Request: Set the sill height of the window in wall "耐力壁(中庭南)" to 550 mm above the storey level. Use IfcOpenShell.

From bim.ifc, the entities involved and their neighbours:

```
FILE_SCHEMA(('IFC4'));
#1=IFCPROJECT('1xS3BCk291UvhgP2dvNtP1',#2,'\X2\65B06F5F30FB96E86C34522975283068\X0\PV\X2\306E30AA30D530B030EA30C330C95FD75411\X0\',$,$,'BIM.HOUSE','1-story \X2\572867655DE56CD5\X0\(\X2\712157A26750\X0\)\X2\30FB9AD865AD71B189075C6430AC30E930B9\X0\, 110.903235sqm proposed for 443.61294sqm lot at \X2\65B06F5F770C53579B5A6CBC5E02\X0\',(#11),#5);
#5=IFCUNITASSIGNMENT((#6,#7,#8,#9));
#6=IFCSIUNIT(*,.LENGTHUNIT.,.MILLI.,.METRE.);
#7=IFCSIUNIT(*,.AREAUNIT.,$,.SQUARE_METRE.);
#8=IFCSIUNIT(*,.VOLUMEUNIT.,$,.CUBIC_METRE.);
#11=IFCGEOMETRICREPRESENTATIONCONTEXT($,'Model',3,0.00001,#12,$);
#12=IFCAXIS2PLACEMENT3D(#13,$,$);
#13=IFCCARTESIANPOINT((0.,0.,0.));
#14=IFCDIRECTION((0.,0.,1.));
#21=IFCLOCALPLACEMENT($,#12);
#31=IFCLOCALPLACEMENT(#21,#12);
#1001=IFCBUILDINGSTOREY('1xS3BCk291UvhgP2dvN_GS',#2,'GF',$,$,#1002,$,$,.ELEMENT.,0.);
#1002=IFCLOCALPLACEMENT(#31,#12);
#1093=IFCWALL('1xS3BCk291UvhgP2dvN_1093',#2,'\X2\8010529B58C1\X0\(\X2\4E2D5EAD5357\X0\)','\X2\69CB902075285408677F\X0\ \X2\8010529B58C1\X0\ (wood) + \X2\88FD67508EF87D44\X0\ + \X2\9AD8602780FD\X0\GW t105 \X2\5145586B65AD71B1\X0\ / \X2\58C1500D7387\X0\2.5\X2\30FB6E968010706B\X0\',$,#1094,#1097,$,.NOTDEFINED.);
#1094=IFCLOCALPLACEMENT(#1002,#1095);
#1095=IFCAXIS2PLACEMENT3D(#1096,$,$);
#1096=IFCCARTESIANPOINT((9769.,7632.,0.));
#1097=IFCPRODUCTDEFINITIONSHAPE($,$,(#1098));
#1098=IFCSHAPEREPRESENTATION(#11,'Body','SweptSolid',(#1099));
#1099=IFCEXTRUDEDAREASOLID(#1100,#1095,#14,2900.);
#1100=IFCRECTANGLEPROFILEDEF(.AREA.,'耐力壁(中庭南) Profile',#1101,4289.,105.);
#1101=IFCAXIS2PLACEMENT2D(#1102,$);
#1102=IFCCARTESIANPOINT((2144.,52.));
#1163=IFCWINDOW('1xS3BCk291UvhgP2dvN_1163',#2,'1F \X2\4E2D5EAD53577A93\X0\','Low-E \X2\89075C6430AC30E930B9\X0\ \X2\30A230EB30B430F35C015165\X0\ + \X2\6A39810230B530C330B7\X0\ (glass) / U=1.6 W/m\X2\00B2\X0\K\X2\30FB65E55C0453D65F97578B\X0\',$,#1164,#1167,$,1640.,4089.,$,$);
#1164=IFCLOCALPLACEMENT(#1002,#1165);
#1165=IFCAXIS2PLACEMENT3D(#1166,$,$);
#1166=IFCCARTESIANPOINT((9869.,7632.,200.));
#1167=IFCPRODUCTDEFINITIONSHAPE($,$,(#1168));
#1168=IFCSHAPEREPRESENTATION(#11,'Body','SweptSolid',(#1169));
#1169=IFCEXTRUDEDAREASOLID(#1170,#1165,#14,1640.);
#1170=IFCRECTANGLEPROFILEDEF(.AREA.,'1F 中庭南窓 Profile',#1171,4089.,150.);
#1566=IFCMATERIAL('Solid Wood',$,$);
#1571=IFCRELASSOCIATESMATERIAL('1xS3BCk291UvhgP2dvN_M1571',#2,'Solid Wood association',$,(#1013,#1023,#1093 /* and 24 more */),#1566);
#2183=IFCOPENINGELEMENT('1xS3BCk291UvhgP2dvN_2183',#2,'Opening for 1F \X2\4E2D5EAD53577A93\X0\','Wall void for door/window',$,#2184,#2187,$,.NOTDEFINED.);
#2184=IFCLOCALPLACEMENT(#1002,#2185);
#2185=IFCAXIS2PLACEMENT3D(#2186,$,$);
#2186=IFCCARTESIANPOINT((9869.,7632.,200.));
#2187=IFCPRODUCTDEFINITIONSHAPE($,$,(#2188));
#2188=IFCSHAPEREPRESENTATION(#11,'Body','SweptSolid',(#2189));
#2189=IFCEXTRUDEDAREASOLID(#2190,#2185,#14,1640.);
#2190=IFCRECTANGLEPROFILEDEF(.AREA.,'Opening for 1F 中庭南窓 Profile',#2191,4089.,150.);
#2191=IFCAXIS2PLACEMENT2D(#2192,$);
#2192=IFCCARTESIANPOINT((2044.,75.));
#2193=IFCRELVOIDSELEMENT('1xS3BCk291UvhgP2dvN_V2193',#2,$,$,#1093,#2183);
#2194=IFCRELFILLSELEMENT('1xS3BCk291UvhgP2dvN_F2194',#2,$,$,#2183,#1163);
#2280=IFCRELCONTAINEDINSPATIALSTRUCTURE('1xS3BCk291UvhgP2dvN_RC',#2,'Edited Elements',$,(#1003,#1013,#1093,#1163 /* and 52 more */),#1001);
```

```python
import numpy as np
import ifcopenshell
import ifcopenshell.api.geometry
import ifcopenshell.geom
import ifcopenshell.util.element
import ifcopenshell.util.placement
import ifcopenshell.util.shape
import ifcopenshell.util.unit

model = ifcopenshell.open("bim.ifc")
unit_scale = ifcopenshell.util.unit.calculate_unit_scale(model)

window = model.by_id(1163)
opening = window.FillsVoids[0].RelatingOpeningElement
storey = ifcopenshell.util.element.get_container(window, ifc_class="IfcBuildingStorey")
level = ifcopenshell.util.placement.get_local_placement(storey.ObjectPlacement)[2, 3]

# The opening's origin need not be at the sill, so measure its lowest point.
shape = ifcopenshell.geom.create_shape(ifcopenshell.geom.settings(), opening)
bottom = ifcopenshell.util.shape.get_shape_bottom_elevation(shape, shape.geometry) / unit_scale
dz = level + 0.55 / unit_scale - bottom

shift = np.array([0.0, 0.0, dz])
# The window is not placed relative to its opening, so move both.
for product in (opening, window):
    matrix = ifcopenshell.util.placement.get_local_placement(product.ObjectPlacement)
    matrix[:3, 3] += shift
    ifcopenshell.api.geometry.edit_object_placement(model, product=product, matrix=matrix, is_si=False)

print(f"moved by {dz * unit_scale:+.3f} m")

model.write("bim_updated.ifc")
```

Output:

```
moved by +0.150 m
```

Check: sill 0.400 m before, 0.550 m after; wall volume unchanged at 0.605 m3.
